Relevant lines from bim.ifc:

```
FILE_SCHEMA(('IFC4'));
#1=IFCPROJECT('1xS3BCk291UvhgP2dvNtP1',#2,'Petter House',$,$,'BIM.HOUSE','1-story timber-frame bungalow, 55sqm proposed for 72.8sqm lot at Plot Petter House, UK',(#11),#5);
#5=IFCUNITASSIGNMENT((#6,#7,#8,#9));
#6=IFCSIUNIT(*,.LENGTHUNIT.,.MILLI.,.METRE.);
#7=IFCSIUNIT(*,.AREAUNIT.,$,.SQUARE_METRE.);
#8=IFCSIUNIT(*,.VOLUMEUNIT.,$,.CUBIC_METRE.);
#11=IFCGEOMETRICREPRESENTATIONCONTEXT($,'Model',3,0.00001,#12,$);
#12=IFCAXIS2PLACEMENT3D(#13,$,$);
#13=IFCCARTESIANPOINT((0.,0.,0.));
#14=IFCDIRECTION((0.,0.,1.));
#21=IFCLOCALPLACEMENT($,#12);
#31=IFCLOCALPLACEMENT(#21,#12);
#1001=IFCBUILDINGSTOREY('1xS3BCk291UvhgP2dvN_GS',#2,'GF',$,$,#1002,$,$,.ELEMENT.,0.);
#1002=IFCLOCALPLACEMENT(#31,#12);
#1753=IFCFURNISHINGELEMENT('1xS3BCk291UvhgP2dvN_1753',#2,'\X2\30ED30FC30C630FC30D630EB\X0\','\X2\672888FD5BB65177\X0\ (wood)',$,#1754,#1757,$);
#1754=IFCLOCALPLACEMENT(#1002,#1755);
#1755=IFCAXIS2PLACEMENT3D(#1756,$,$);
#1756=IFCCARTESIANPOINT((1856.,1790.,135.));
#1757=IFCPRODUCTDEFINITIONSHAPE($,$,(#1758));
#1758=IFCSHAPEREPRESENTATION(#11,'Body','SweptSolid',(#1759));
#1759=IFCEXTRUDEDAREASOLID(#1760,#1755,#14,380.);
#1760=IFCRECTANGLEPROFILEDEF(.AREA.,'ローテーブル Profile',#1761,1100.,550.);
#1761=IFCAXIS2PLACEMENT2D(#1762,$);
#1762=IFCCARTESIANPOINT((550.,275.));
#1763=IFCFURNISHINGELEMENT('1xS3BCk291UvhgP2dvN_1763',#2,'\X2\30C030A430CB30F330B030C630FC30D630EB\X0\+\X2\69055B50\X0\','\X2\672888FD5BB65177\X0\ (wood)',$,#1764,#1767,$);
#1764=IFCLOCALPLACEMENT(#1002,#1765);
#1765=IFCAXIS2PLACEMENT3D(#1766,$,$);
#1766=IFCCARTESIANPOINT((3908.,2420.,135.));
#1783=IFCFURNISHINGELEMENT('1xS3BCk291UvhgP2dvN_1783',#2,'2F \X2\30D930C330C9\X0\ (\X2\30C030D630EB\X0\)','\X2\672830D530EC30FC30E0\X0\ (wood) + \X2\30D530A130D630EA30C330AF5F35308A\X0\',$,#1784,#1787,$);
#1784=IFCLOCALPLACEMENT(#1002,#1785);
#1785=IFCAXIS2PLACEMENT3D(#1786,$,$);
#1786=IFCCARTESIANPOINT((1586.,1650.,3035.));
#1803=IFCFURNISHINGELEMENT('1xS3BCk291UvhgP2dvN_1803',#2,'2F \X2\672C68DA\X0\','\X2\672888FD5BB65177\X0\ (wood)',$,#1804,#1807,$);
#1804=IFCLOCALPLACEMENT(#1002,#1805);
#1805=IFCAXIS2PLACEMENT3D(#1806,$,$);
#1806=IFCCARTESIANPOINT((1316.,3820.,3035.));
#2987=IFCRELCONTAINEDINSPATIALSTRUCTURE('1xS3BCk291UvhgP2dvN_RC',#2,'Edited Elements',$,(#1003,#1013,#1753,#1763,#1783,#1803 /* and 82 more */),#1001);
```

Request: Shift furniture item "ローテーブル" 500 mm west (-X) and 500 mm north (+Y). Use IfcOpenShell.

```python
import ifcopenshell
import ifcopenshell.api.geometry
import ifcopenshell.util.placement
import ifcopenshell.util.unit

model = ifcopenshell.open("bim.ifc")
unit_scale = ifcopenshell.util.unit.calculate_unit_scale(model)

item = model.by_guid("1xS3BCk291UvhgP2dvN_1753")
matrix = ifcopenshell.util.placement.get_local_placement(item.ObjectPlacement)
matrix[0, 3] -= 0.5 / unit_scale
matrix[1, 3] += 0.5 / unit_scale
ifcopenshell.api.geometry.edit_object_placement(model, product=item, matrix=matrix, is_si=False)

print(ifcopenshell.util.placement.get_local_placement(item.ObjectPlacement).round(3) + 0.0)

model.write("bim_updated.ifc")
```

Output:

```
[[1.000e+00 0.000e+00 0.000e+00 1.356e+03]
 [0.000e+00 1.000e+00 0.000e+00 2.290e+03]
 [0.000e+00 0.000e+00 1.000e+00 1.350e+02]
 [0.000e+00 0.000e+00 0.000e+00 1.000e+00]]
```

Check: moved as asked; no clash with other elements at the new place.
